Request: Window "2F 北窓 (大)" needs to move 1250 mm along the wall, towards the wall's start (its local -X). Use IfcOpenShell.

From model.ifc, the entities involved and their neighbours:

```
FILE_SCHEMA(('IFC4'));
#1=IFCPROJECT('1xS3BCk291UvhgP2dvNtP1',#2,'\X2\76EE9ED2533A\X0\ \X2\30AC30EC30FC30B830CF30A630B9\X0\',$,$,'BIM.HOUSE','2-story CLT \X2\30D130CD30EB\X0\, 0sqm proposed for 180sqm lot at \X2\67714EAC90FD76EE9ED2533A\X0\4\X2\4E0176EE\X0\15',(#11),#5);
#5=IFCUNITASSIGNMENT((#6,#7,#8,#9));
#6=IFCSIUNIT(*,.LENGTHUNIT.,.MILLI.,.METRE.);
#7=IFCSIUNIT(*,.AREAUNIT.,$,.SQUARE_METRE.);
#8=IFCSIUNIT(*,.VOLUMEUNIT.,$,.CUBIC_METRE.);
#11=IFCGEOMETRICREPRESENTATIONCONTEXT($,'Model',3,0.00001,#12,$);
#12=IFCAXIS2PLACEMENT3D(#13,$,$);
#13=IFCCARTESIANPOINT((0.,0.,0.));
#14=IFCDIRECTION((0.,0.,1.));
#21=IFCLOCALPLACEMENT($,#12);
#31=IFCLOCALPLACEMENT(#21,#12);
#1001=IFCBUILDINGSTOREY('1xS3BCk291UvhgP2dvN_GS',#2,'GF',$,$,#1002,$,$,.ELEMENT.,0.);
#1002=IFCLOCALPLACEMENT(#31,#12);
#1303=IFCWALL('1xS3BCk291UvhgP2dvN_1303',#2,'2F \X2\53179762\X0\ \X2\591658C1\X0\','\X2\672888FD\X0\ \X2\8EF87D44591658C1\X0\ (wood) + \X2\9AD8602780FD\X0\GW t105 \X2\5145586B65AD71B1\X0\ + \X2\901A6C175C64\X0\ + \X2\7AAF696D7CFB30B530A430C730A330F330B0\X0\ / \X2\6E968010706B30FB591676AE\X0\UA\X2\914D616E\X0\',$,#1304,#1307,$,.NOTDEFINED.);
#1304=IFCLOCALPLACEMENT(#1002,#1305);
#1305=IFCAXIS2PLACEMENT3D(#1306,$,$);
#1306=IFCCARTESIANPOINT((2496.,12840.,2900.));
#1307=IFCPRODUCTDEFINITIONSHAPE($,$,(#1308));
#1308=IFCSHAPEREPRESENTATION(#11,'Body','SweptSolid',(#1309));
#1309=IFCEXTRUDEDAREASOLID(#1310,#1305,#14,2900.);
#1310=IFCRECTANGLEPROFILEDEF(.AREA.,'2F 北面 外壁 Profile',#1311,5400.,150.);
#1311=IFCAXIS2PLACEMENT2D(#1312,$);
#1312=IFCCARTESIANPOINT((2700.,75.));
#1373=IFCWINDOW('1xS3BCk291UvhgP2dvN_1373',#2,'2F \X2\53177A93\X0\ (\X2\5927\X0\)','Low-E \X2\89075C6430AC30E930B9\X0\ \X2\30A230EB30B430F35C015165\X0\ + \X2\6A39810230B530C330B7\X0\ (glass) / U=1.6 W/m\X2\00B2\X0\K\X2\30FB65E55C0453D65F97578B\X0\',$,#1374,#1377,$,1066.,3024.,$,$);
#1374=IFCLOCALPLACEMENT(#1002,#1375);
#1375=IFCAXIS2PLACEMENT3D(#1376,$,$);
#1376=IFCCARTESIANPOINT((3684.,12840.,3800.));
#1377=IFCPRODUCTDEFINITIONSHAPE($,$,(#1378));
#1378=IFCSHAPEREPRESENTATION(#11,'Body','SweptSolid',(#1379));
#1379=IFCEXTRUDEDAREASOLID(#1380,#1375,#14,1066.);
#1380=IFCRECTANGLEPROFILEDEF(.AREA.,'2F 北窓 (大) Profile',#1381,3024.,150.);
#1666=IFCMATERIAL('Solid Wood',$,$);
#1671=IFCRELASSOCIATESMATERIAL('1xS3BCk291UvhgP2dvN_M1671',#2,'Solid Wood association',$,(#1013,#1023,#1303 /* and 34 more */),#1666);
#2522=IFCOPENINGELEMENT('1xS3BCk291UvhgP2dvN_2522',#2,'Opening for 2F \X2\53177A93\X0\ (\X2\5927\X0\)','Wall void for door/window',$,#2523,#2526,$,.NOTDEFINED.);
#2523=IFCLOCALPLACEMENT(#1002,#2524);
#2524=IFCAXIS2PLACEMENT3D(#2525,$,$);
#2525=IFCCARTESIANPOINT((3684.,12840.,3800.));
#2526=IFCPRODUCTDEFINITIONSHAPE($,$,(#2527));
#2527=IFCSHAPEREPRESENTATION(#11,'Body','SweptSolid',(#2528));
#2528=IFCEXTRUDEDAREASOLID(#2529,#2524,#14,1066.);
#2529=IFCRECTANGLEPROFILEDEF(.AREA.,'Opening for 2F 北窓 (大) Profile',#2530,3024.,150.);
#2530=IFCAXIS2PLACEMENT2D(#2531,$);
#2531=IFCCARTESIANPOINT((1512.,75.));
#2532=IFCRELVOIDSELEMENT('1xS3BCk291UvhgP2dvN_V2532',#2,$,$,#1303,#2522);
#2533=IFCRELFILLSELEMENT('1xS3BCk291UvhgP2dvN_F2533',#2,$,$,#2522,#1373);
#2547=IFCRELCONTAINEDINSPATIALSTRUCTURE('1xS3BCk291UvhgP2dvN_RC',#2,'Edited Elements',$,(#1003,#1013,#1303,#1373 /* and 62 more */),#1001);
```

```python
import ifcopenshell
import ifcopenshell.api.geometry
import ifcopenshell.util.placement
import ifcopenshell.util.unit

model = ifcopenshell.open("model.ifc")
unit_scale = ifcopenshell.util.unit.calculate_unit_scale(model)

window = model.by_guid("1xS3BCk291UvhgP2dvN_1373")
opening = window.FillsVoids[0].RelatingOpeningElement
wall = opening.VoidsElements[0].RelatingBuildingElement

wall_matrix = ifcopenshell.util.placement.get_local_placement(wall.ObjectPlacement)
shift = wall_matrix[:3, 0] * -1.25 / unit_scale
before = ifcopenshell.util.placement.get_local_placement(window.ObjectPlacement)[:3, 3].copy()

# The window is not placed relative to its opening, so move both.
for product in (opening, window):
    matrix = ifcopenshell.util.placement.get_local_placement(product.ObjectPlacement)
    matrix[:3, 3] += shift
    ifcopenshell.api.geometry.edit_object_placement(model, product=product, matrix=matrix, is_si=False)

after = ifcopenshell.util.placement.get_local_placement(window.ObjectPlacement)[:3, 3]
print("window moved by", (after - before).round(3) + 0.0)

model.write("model_v2.ifc")
```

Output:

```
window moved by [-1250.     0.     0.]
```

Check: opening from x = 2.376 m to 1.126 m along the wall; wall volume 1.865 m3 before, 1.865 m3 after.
